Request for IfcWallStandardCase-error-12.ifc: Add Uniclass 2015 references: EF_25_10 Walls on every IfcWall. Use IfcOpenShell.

First a look at what the model holds.

```python
import ifcopenshell

model = ifcopenshell.open("IfcWallStandardCase-error-12.ifc")
print(model.schema)
print("classifications:", [c.Name for c in model.by_type("IfcClassification")])
for ifc_class in ("IfcDoor", "IfcRoof", "IfcStair", "IfcWall", "IfcWindow"):
    print(ifc_class, len(model.by_type(ifc_class)))
```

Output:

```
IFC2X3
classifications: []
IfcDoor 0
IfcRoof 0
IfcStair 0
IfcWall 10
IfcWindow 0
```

```python
import ifcopenshell
import ifcopenshell.api.classification

model = ifcopenshell.open("IfcWallStandardCase-error-12.ifc")

# IFC2X3 requires Source and Edition and has no link from the project to the system.
system = model.create_entity("IfcClassification", Source="NBS", Edition="2015", Name="Uniclass 2015")

codes = {
    "IfcWall": ("EF_25_10", "Walls"),
}
for ifc_class, (code, name) in codes.items():
    products = model.by_type(ifc_class)
    ifcopenshell.api.classification.add_reference(
        model, products=products, classification=system, identification=code, name=name
    )
    print(code, len(products))

model.write("IfcWallStandardCase-error-12-out.ifc")
```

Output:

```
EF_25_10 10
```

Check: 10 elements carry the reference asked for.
